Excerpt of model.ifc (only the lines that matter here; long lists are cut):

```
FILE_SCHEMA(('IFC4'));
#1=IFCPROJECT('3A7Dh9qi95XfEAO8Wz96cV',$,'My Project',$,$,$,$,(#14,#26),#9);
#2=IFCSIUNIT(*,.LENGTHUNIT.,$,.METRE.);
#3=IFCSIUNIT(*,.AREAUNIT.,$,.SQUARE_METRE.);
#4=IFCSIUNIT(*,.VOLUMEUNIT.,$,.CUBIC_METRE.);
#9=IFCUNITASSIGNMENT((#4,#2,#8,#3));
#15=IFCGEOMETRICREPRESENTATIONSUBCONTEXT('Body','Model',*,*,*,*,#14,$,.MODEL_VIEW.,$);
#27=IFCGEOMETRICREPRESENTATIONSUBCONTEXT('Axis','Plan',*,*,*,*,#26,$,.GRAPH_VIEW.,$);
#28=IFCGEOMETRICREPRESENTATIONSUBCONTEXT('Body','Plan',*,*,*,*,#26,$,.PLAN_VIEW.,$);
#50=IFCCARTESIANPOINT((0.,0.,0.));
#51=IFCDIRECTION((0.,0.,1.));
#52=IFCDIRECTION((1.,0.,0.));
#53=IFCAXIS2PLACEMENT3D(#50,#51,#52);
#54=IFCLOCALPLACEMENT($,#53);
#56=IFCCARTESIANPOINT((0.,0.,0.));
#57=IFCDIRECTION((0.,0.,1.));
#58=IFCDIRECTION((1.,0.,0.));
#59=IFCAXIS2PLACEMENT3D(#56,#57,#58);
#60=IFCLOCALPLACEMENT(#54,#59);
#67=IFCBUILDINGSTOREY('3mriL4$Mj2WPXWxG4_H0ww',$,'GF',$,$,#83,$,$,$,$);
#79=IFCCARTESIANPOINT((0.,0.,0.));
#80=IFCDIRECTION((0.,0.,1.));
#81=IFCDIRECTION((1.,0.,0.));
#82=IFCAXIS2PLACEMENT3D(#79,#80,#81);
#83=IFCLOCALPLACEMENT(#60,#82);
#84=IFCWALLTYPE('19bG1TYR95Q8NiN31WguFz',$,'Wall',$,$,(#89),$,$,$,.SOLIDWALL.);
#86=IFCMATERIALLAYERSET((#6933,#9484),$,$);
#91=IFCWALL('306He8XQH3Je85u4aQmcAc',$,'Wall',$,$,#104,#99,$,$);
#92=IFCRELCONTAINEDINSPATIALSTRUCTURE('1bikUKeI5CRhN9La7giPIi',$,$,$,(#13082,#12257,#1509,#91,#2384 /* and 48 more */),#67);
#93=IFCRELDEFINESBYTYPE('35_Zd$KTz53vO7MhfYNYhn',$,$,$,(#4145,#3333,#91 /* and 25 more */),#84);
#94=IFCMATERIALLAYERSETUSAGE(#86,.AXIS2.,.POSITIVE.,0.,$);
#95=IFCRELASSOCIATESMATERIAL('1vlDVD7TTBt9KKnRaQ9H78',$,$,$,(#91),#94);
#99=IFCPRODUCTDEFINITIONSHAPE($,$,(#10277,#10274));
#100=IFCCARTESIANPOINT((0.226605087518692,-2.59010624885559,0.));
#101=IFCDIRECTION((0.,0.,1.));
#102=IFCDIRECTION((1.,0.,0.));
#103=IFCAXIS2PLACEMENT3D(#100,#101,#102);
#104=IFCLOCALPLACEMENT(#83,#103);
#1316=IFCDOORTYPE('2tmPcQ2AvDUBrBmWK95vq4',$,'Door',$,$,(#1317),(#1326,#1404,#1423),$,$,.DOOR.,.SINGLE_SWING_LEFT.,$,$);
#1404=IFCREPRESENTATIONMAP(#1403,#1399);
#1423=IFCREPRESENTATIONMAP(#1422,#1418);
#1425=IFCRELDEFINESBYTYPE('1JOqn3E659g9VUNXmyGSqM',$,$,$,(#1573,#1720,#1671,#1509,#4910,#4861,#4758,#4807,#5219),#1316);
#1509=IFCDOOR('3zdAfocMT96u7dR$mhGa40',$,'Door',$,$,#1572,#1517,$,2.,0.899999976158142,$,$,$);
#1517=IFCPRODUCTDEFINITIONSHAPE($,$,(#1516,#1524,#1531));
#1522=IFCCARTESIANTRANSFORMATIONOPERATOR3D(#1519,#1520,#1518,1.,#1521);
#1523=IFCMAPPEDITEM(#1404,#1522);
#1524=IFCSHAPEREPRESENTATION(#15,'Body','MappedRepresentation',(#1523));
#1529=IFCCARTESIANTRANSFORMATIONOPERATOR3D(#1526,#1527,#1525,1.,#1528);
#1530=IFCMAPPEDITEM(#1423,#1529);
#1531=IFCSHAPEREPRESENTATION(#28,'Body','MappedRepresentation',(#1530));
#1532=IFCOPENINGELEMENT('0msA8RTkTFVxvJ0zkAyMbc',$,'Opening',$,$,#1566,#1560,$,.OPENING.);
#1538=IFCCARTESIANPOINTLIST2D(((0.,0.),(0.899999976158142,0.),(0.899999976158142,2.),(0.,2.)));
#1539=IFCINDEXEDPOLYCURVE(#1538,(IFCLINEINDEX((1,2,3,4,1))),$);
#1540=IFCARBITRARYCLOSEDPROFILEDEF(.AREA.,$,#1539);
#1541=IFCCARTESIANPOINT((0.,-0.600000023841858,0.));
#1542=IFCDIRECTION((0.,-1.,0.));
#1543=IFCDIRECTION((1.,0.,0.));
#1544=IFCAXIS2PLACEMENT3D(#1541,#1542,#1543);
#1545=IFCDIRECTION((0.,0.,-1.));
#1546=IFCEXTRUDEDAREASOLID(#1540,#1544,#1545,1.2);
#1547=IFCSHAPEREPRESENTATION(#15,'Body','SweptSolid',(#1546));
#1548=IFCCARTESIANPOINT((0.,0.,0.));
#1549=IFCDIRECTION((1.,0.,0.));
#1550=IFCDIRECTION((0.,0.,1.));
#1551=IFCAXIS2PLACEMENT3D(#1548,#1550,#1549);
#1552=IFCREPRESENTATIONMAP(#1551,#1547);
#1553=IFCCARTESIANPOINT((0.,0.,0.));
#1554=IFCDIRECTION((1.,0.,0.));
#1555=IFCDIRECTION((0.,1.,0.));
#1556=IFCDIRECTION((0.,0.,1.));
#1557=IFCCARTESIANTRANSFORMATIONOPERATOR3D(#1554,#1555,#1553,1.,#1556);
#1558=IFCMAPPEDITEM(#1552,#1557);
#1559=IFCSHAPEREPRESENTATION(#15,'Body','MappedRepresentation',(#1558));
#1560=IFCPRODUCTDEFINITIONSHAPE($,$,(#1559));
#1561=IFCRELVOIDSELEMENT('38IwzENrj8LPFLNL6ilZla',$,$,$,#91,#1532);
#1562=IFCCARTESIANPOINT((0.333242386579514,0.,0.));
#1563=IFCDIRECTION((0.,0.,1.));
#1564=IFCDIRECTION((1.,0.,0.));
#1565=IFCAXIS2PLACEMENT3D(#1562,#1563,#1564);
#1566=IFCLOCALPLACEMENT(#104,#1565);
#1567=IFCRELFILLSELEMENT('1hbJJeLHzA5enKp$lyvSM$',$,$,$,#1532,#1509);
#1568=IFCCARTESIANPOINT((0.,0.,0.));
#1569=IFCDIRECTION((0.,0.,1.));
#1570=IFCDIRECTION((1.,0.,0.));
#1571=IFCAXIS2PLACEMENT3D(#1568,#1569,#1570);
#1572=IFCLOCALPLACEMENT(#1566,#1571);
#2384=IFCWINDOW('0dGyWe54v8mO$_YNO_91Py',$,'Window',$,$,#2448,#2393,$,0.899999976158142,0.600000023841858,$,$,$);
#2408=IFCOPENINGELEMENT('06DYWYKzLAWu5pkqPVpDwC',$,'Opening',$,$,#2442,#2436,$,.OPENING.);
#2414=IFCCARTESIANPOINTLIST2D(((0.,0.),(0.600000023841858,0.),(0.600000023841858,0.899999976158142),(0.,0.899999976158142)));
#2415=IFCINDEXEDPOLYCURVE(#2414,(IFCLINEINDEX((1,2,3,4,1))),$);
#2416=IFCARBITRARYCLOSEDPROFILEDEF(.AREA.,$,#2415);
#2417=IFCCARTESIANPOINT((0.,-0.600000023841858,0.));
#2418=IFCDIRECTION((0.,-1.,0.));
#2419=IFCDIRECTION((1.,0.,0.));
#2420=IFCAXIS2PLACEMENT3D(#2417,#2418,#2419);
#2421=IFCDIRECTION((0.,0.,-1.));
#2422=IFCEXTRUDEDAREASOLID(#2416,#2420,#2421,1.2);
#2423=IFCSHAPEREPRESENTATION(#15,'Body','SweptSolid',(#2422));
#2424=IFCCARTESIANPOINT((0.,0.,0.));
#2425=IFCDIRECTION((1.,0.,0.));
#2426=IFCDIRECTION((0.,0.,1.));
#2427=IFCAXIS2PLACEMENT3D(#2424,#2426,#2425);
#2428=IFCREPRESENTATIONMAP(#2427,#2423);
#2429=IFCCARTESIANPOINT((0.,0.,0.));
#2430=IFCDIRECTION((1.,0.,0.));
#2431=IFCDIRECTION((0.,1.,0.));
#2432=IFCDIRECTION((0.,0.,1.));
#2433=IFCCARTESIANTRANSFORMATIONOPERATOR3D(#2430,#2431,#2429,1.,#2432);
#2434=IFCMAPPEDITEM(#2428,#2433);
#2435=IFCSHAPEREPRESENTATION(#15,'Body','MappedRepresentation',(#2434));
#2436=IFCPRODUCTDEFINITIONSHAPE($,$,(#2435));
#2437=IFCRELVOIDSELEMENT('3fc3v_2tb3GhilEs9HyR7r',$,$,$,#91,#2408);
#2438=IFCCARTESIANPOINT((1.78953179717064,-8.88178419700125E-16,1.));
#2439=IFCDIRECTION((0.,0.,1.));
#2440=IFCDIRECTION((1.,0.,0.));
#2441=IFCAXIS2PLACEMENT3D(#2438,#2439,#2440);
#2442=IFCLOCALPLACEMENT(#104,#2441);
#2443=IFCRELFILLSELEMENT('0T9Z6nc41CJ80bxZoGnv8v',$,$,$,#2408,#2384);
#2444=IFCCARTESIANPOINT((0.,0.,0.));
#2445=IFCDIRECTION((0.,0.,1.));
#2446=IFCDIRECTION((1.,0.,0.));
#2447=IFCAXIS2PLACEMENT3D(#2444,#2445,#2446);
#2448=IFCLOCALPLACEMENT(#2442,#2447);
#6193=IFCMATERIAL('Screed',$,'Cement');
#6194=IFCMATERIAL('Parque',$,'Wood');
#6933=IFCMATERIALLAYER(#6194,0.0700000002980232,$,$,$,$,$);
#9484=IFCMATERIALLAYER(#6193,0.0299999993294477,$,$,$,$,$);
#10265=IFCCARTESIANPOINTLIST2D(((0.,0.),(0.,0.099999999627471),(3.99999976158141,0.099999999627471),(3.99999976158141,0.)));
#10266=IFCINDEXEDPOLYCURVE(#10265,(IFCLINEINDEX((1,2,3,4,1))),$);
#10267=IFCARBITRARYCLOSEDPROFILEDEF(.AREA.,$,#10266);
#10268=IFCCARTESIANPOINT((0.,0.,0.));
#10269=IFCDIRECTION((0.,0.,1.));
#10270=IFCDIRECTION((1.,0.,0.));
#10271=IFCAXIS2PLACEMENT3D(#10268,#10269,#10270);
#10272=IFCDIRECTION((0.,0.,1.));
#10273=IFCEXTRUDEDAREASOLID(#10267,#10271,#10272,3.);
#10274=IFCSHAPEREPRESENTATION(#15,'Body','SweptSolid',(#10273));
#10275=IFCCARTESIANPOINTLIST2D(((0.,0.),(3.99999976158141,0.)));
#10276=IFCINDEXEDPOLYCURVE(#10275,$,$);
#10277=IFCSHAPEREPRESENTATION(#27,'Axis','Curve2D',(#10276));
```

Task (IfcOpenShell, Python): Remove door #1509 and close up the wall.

```python
import ifcopenshell
import ifcopenshell.api.feature
import ifcopenshell.api.root
import ifcopenshell.geom
import ifcopenshell.util.shape

model = ifcopenshell.open("model.ifc")
settings = ifcopenshell.geom.settings()


def volume(element):
    """Net volume in cubic metres, openings subtracted."""
    shape = ifcopenshell.geom.create_shape(settings, element)
    return ifcopenshell.util.shape.get_volume(shape.geometry)


door = model.by_id(1509)
opening = door.FillsVoids[0].RelatingOpeningElement
wall = opening.VoidsElements[0].RelatingBuildingElement
before = volume(wall)

ifcopenshell.api.root.remove_product(model, product=door)
ifcopenshell.api.feature.remove_feature(model, feature=opening)

after = volume(wall)

print(f"wall volume {before:.3f} -> {after:.3f} m3")

model.write("model_updated.ifc")
```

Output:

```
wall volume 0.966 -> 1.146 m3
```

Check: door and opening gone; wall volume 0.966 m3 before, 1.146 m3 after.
